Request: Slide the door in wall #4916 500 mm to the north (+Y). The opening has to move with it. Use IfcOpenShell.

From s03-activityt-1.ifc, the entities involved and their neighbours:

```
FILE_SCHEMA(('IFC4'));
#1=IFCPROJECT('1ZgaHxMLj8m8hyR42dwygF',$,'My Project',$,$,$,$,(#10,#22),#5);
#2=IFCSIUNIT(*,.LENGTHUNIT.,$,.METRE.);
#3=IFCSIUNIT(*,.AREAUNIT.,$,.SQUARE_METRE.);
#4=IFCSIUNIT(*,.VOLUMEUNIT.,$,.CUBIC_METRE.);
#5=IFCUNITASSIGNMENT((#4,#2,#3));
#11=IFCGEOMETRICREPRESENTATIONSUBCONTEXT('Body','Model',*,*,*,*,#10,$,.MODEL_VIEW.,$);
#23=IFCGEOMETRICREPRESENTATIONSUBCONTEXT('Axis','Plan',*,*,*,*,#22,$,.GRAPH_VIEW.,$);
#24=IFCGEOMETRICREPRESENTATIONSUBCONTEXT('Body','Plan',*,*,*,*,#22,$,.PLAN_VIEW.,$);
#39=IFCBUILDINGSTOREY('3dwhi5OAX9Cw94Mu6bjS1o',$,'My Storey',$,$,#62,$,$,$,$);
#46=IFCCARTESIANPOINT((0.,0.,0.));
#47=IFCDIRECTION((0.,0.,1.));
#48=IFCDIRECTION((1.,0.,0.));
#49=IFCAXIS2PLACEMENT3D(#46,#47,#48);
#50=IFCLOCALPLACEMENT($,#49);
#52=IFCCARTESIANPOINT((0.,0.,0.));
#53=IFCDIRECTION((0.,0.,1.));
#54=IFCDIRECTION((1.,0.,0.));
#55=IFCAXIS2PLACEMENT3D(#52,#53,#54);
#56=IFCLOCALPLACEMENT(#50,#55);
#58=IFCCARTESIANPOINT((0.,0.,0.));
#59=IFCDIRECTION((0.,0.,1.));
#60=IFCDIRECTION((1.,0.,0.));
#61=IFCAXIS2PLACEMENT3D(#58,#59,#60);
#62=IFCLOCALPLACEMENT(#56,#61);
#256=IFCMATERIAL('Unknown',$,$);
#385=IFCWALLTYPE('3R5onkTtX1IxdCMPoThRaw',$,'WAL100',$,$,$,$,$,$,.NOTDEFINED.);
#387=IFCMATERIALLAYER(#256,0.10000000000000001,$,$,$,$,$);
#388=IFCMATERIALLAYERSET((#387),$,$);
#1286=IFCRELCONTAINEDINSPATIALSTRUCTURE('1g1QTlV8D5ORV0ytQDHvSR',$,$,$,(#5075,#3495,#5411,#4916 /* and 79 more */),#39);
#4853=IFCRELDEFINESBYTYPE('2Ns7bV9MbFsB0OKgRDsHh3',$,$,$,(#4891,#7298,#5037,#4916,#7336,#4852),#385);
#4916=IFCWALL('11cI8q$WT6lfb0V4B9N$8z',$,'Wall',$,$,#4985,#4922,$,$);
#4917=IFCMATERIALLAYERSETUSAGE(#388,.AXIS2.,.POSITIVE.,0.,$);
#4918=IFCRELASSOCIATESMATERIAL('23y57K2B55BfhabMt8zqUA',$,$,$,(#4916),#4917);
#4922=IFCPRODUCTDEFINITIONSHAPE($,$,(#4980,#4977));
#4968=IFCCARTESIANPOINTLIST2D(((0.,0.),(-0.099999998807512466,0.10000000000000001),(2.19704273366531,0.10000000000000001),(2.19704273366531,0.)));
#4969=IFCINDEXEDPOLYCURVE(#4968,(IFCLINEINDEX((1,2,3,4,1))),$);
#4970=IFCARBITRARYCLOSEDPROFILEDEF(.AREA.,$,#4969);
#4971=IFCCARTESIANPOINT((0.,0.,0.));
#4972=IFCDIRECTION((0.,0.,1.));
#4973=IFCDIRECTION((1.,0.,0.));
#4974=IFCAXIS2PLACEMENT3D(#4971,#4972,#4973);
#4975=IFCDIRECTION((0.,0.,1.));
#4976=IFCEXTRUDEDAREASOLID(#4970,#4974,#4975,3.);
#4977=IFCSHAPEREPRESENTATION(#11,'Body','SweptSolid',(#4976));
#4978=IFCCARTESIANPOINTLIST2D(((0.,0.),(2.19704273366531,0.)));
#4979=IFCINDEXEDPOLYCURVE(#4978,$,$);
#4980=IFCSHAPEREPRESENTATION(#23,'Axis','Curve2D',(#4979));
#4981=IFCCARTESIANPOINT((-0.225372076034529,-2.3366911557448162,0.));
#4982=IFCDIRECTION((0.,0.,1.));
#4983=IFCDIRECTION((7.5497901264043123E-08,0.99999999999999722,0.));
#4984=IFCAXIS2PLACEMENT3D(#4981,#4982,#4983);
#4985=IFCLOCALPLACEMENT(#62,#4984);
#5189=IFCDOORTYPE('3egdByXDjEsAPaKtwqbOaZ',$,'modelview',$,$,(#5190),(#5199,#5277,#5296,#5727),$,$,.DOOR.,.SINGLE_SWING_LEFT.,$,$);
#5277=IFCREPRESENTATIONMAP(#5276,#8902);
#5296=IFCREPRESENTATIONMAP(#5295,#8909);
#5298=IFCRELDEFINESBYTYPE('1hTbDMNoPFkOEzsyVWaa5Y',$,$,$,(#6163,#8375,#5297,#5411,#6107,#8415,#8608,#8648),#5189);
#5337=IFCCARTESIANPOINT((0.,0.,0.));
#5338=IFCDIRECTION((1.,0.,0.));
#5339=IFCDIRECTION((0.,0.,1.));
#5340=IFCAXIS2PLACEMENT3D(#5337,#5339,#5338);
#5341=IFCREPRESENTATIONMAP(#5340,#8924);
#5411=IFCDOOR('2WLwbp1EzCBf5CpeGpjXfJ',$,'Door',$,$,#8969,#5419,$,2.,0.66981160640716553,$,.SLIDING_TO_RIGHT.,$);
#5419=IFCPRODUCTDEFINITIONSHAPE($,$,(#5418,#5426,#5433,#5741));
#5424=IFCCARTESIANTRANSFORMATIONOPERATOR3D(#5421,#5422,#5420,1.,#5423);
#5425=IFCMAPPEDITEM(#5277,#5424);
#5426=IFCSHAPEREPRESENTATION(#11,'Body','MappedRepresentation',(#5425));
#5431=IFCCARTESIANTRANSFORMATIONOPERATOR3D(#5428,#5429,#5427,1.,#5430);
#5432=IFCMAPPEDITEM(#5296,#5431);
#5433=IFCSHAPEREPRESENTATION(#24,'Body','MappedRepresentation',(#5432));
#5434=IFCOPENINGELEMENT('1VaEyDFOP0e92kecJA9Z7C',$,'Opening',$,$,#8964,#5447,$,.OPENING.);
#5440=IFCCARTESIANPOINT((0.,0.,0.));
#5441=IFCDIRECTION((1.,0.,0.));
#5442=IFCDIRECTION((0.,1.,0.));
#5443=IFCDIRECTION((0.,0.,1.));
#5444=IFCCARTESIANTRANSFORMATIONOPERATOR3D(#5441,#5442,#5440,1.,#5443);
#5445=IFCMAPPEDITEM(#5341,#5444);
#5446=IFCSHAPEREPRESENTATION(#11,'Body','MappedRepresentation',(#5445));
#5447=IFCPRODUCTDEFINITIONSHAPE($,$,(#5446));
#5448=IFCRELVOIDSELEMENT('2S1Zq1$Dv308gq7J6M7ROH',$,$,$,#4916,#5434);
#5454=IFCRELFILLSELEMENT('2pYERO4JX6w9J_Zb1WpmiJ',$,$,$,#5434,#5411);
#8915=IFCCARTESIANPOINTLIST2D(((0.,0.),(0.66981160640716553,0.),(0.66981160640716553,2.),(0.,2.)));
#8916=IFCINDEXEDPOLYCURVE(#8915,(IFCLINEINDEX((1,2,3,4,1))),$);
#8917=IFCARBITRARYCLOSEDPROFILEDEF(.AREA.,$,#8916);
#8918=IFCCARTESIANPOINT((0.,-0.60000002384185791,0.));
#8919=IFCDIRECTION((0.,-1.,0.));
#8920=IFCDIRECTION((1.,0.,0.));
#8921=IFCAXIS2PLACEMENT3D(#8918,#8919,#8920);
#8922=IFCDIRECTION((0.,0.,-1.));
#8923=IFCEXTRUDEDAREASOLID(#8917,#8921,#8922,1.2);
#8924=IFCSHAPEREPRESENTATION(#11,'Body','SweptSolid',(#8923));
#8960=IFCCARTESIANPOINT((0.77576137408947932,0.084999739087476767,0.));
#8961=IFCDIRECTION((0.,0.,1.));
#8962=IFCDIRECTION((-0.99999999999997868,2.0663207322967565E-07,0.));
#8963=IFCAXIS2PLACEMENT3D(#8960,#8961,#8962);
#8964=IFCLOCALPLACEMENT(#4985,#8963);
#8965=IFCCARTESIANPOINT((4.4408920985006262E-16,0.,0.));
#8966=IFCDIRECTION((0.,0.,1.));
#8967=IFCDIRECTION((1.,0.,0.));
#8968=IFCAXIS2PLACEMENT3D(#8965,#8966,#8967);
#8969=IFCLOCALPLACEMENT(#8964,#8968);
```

```python
import ifcopenshell
import ifcopenshell.api.geometry
import ifcopenshell.util.placement
import ifcopenshell.util.unit

model = ifcopenshell.open("s03-activityt-1.ifc")
unit_scale = ifcopenshell.util.unit.calculate_unit_scale(model)

door = model.by_guid("2WLwbp1EzCBf5CpeGpjXfJ")
opening = door.FillsVoids[0].RelatingOpeningElement
wall = opening.VoidsElements[0].RelatingBuildingElement

wall_matrix = ifcopenshell.util.placement.get_local_placement(wall.ObjectPlacement)
shift = wall_matrix[:3, 0] * 0.5 / unit_scale
before = ifcopenshell.util.placement.get_local_placement(door.ObjectPlacement)[:3, 3].copy()

# The door is placed relative to its opening, so it follows when the opening moves.
matrix = ifcopenshell.util.placement.get_local_placement(opening.ObjectPlacement)
matrix[:3, 3] += shift
ifcopenshell.api.geometry.edit_object_placement(
    model, product=opening, matrix=matrix, is_si=False, should_transform_children=True
)

after = ifcopenshell.util.placement.get_local_placement(door.ObjectPlacement)[:3, 3]
print("door moved by", (after - before).round(3) + 0.0)

model.write("s03-activityt-1_edited.ifc")
```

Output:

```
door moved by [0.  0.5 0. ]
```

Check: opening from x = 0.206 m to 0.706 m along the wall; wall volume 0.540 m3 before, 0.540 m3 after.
